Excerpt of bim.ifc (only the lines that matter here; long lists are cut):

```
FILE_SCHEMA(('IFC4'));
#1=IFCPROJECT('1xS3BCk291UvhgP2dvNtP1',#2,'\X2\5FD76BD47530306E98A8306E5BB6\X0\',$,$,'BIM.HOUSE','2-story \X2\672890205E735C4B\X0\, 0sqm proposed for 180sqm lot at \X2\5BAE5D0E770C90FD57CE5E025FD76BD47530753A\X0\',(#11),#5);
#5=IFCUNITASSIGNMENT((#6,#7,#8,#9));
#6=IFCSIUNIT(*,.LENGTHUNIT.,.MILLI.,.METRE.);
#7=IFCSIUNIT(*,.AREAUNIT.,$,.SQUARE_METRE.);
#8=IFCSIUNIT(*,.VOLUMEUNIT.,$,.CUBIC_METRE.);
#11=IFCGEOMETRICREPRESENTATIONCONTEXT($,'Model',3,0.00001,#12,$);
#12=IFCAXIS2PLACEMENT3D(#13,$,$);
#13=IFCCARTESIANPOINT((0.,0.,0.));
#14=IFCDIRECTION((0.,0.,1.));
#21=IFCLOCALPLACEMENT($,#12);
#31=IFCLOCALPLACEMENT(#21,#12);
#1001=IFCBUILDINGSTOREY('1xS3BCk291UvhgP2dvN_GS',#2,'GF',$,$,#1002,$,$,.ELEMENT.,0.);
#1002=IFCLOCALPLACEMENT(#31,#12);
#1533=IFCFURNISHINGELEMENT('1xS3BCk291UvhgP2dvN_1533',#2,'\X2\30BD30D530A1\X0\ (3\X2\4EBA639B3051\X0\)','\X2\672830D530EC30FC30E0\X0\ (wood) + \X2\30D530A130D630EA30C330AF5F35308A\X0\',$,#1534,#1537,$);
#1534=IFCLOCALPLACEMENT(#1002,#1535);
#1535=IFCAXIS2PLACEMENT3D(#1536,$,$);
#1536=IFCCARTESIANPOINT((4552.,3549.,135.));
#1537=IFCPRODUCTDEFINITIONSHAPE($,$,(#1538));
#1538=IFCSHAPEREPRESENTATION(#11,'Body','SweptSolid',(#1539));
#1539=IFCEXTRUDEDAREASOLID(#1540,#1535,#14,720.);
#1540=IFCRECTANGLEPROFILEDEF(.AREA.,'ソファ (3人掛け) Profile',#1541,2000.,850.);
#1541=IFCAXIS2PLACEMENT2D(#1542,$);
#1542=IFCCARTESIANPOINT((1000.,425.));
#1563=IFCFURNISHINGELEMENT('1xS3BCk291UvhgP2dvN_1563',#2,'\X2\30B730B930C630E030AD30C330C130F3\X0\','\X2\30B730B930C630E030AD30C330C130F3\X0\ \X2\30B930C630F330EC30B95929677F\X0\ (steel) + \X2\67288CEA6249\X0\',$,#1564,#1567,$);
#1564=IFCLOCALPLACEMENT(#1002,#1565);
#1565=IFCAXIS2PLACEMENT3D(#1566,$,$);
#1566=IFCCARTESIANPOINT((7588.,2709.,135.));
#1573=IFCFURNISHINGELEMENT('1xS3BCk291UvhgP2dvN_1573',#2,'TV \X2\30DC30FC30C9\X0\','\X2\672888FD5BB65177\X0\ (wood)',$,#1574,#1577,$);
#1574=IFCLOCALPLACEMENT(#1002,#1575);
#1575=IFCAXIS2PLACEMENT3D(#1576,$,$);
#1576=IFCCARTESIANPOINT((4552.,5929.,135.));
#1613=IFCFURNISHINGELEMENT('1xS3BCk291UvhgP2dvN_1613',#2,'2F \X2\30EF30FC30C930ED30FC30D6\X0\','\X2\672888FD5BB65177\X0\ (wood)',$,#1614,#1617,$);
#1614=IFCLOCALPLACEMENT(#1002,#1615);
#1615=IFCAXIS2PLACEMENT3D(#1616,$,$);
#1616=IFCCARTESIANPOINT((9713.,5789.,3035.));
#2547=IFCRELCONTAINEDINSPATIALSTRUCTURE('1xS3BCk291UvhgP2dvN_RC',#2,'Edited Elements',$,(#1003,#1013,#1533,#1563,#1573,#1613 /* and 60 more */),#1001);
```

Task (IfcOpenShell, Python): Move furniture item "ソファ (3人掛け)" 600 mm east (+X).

```python
import ifcopenshell
import ifcopenshell.api.geometry
import ifcopenshell.util.placement
import ifcopenshell.util.unit

model = ifcopenshell.open("bim.ifc")
unit_scale = ifcopenshell.util.unit.calculate_unit_scale(model)

item = model.by_id(1533)
matrix = ifcopenshell.util.placement.get_local_placement(item.ObjectPlacement)
matrix[0, 3] += 0.6 / unit_scale
ifcopenshell.api.geometry.edit_object_placement(model, product=item, matrix=matrix, is_si=False)

print(ifcopenshell.util.placement.get_local_placement(item.ObjectPlacement).round(3) + 0.0)

model.write("bim_updated.ifc")
```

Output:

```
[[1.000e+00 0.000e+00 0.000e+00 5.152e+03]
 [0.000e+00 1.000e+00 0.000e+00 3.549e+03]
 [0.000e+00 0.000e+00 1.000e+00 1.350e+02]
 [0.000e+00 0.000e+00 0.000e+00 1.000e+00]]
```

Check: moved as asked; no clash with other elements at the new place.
